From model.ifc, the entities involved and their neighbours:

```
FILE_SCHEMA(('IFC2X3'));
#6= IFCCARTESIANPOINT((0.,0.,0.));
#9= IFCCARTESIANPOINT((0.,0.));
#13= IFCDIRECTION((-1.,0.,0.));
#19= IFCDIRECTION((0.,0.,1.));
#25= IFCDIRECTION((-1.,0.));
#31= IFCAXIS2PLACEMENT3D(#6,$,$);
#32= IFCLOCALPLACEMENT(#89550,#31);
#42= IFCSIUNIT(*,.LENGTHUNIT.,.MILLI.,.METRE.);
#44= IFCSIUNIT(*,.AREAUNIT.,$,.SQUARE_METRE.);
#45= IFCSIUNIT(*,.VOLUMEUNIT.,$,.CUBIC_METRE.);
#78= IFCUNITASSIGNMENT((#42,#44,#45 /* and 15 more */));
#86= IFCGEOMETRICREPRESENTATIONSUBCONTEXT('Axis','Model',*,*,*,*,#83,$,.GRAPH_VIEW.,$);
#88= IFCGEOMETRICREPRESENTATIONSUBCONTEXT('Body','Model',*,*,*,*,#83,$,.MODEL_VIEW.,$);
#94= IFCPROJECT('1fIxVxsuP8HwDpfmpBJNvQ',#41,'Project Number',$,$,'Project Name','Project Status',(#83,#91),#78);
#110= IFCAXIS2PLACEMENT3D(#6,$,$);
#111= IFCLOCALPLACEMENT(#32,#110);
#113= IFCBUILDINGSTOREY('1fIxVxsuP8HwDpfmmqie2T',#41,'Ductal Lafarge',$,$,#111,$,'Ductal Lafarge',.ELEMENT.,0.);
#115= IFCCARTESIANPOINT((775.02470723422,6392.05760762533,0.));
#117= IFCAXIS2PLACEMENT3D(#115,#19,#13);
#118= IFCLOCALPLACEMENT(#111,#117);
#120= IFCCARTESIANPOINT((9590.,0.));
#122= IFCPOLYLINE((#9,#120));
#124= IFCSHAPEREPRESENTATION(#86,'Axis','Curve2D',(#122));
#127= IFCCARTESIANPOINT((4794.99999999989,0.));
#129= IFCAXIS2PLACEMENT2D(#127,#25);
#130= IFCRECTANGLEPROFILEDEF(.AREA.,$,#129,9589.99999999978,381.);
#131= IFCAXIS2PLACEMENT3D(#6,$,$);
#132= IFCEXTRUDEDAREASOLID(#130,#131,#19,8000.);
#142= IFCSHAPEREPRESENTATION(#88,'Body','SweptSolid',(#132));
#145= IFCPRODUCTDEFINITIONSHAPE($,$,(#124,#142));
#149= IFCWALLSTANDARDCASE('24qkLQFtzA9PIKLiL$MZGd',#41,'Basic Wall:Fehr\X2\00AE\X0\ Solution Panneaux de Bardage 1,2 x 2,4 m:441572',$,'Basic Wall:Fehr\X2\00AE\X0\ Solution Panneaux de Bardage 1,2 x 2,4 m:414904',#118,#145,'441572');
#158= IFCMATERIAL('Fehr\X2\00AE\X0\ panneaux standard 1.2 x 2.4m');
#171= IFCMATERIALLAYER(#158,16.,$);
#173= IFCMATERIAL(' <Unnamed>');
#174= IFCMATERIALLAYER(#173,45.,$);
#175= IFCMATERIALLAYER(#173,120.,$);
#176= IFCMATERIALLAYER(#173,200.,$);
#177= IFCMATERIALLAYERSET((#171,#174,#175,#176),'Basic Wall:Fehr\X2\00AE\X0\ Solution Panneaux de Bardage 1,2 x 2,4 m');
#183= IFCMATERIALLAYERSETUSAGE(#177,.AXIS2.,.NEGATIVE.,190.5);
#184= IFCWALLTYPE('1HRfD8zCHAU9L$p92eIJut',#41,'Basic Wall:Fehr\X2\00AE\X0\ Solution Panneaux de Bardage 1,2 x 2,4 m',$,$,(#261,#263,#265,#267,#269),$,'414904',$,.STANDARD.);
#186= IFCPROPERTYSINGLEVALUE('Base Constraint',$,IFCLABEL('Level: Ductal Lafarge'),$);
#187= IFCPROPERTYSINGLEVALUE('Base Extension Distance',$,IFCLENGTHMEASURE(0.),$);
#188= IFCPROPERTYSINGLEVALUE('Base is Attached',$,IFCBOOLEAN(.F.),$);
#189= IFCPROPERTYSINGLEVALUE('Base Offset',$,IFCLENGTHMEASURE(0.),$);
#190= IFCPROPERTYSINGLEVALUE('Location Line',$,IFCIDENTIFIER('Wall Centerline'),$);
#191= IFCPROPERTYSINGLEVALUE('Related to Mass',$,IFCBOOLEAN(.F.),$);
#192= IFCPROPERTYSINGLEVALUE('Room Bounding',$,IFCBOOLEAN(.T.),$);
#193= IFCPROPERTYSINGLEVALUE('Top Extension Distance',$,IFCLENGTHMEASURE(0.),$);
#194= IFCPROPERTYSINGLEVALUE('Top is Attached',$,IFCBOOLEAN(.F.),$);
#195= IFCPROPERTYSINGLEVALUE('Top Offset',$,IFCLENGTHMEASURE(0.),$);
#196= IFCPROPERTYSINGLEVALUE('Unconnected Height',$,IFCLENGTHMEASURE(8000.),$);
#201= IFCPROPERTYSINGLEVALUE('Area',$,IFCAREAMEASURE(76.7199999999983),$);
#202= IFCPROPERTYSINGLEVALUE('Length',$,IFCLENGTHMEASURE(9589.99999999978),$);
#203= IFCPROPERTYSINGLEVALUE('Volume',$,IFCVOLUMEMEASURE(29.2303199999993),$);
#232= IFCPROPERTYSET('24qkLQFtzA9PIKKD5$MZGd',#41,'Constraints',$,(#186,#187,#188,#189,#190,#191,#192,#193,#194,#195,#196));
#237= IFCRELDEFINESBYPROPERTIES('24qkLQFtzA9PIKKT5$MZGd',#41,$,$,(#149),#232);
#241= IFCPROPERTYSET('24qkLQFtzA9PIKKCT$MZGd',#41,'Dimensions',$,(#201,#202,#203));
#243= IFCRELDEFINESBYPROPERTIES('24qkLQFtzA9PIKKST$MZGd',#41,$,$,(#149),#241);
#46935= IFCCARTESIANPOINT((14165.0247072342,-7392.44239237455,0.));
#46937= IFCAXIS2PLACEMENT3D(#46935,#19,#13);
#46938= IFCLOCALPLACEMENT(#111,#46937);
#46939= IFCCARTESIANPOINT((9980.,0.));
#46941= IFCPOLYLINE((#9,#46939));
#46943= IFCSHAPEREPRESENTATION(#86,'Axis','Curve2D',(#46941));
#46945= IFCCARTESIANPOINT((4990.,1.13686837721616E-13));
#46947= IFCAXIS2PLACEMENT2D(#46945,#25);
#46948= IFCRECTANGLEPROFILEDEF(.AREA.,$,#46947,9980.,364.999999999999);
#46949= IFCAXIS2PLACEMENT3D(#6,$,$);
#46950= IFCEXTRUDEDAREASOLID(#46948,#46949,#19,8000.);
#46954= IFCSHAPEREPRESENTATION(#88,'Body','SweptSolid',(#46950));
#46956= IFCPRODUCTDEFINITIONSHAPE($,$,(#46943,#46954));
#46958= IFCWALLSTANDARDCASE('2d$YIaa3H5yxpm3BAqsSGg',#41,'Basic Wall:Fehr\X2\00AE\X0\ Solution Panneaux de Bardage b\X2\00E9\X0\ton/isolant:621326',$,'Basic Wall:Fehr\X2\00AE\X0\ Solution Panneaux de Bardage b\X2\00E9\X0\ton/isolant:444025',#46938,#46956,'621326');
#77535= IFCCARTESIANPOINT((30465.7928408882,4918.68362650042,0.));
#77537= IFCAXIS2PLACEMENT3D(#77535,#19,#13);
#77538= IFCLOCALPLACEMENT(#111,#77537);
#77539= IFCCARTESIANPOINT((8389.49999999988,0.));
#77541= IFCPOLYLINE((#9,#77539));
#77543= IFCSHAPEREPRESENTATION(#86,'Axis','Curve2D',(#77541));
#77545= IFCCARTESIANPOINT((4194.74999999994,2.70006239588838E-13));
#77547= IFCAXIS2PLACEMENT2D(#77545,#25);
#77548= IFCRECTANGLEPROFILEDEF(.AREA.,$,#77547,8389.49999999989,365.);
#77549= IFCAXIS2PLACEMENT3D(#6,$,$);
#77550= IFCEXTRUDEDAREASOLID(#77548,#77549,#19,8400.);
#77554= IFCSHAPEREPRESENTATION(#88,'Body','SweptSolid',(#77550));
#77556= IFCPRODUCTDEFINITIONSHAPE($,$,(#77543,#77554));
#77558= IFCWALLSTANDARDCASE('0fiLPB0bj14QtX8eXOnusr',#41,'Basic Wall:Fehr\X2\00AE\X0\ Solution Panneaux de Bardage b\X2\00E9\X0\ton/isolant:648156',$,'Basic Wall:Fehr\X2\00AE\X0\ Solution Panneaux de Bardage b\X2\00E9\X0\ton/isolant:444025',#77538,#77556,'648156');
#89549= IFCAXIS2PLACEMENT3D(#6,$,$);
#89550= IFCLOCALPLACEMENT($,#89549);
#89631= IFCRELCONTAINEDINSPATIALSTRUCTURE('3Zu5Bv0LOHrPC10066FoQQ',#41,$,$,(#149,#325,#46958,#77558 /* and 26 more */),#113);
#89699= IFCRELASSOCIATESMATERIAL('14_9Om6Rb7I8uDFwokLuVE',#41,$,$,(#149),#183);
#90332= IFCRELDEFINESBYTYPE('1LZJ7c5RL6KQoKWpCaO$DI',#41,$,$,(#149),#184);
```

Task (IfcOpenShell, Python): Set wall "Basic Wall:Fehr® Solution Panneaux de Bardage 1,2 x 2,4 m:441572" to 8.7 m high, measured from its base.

```python
import ifcopenshell
import ifcopenshell.api.pset
import ifcopenshell.geom
import ifcopenshell.util.element
import ifcopenshell.util.representation
import ifcopenshell.util.shape
import ifcopenshell.util.unit

model = ifcopenshell.open("model.ifc")
unit_scale = ifcopenshell.util.unit.calculate_unit_scale(model)
area_scale = ifcopenshell.util.unit.calculate_unit_scale(model, "AREAUNIT")
volume_scale = ifcopenshell.util.unit.calculate_unit_scale(model, "VOLUMEUNIT")
settings = ifcopenshell.geom.settings()


def volume(element):
    """Net volume in cubic metres, openings subtracted."""
    shape = ifcopenshell.geom.create_shape(settings, element)
    return ifcopenshell.util.shape.get_volume(shape.geometry)


wall = model.by_guid("24qkLQFtzA9PIKLiL$MZGd")
before = volume(wall)

body = ifcopenshell.util.representation.get_representation(wall, "Model", "Body")
solid = body.Items[0]
old_height = solid.Depth
solid.Depth = 8.7 / unit_scale
after = volume(wall)
thickness = 0.381  # wall thickness in metres

# Update the stored height, areas and volumes.
pset = model.by_id(ifcopenshell.util.element.get_pset(wall, "Constraints", should_inherit=False)["id"])
ifcopenshell.api.pset.edit_pset(model, pset=pset, properties={
    "Unconnected Height": model.create_entity("IfcLengthMeasure", solid.Depth),
})
pset = model.by_id(ifcopenshell.util.element.get_pset(wall, "Dimensions", should_inherit=False)["id"])
ifcopenshell.api.pset.edit_pset(model, pset=pset, properties={
    "Area": model.create_entity("IfcAreaMeasure", after / thickness / area_scale),
    "Volume": model.create_entity("IfcVolumeMeasure", after / volume_scale),
})

print(f"height {old_height:g} -> {solid.Depth:g}, volume {before:.3f} -> {after:.3f} m3")

model.write("model_updated.ifc")
```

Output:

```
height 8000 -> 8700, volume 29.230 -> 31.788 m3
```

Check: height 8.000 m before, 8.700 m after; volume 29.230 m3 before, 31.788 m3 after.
